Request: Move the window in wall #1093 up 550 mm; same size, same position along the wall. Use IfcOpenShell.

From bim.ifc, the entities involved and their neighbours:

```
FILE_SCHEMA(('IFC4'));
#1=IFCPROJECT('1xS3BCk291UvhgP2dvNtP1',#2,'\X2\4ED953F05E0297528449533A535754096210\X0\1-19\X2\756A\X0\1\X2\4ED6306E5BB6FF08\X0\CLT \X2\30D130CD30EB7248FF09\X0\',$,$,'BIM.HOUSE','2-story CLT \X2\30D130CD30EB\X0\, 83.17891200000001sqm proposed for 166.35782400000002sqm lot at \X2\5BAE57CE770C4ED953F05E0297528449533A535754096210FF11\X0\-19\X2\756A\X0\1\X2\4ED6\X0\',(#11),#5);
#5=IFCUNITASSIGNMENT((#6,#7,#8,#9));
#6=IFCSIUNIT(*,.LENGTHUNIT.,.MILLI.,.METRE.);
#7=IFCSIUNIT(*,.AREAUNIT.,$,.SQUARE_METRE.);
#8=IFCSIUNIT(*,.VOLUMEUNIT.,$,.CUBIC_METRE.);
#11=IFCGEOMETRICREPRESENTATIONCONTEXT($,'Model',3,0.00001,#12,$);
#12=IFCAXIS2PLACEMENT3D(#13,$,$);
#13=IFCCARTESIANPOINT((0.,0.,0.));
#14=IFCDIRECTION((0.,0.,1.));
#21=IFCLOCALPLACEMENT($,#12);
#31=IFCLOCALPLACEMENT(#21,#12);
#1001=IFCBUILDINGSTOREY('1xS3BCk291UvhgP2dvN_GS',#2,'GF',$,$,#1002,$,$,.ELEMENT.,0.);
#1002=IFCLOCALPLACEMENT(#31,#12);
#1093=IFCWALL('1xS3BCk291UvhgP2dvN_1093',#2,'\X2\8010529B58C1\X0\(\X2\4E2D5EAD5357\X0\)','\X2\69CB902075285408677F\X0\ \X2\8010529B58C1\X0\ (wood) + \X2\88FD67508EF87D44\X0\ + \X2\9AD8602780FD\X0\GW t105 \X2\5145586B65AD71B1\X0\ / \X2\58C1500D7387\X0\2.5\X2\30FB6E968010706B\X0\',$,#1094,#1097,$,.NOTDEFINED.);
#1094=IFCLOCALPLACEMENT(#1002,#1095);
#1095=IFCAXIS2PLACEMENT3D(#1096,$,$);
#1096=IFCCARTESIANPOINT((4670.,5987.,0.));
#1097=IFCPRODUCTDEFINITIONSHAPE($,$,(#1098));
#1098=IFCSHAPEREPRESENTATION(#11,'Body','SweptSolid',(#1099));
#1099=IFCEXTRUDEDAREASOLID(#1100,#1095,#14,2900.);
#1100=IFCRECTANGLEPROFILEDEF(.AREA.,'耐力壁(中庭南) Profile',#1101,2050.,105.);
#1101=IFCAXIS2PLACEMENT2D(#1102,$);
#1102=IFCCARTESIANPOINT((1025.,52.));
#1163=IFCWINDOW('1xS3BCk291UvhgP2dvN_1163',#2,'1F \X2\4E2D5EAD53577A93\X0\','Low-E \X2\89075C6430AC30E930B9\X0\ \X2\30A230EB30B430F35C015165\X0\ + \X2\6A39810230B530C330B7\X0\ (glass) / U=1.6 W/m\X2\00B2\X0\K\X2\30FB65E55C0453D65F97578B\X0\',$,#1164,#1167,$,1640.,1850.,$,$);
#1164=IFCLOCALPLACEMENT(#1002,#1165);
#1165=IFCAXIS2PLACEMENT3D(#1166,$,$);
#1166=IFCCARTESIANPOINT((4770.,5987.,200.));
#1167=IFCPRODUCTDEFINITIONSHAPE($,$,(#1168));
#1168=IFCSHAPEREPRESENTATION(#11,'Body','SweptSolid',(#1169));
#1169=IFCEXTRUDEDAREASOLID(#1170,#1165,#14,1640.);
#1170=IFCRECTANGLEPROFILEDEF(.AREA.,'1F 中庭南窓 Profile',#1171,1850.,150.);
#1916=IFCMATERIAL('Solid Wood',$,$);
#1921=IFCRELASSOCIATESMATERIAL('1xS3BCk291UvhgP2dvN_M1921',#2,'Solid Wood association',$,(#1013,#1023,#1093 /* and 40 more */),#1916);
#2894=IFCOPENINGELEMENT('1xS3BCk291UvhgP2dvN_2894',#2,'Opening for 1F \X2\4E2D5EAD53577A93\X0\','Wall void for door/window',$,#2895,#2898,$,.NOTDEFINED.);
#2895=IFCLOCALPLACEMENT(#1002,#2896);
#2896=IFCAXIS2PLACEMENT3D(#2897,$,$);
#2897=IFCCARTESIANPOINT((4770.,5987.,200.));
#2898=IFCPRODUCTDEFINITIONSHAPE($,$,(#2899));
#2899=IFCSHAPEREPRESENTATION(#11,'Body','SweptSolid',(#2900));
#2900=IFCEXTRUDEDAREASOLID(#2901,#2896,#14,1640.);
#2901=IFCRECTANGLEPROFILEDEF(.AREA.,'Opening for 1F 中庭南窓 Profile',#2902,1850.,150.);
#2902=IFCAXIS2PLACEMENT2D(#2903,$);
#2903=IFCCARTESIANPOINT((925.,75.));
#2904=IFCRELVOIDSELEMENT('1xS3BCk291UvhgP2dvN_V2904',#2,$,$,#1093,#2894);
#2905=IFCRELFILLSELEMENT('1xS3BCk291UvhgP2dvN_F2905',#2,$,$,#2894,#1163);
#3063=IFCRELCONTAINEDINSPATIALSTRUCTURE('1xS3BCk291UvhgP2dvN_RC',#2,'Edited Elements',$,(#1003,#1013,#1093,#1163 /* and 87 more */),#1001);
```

```python
import numpy as np
import ifcopenshell
import ifcopenshell.api.geometry
import ifcopenshell.util.placement
import ifcopenshell.util.unit

model = ifcopenshell.open("bim.ifc")
unit_scale = ifcopenshell.util.unit.calculate_unit_scale(model)

window = model.by_guid("1xS3BCk291UvhgP2dvN_1163")
opening = window.FillsVoids[0].RelatingOpeningElement
dz = 0.55 / unit_scale

shift = np.array([0.0, 0.0, dz])
# The window is not placed relative to its opening, so move both.
for product in (opening, window):
    matrix = ifcopenshell.util.placement.get_local_placement(product.ObjectPlacement)
    matrix[:3, 3] += shift
    ifcopenshell.api.geometry.edit_object_placement(model, product=product, matrix=matrix, is_si=False)

print(f"moved by {dz * unit_scale:+.3f} m")

model.write("bim-out.ifc")
```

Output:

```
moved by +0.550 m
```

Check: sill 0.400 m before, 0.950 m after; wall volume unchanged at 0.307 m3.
